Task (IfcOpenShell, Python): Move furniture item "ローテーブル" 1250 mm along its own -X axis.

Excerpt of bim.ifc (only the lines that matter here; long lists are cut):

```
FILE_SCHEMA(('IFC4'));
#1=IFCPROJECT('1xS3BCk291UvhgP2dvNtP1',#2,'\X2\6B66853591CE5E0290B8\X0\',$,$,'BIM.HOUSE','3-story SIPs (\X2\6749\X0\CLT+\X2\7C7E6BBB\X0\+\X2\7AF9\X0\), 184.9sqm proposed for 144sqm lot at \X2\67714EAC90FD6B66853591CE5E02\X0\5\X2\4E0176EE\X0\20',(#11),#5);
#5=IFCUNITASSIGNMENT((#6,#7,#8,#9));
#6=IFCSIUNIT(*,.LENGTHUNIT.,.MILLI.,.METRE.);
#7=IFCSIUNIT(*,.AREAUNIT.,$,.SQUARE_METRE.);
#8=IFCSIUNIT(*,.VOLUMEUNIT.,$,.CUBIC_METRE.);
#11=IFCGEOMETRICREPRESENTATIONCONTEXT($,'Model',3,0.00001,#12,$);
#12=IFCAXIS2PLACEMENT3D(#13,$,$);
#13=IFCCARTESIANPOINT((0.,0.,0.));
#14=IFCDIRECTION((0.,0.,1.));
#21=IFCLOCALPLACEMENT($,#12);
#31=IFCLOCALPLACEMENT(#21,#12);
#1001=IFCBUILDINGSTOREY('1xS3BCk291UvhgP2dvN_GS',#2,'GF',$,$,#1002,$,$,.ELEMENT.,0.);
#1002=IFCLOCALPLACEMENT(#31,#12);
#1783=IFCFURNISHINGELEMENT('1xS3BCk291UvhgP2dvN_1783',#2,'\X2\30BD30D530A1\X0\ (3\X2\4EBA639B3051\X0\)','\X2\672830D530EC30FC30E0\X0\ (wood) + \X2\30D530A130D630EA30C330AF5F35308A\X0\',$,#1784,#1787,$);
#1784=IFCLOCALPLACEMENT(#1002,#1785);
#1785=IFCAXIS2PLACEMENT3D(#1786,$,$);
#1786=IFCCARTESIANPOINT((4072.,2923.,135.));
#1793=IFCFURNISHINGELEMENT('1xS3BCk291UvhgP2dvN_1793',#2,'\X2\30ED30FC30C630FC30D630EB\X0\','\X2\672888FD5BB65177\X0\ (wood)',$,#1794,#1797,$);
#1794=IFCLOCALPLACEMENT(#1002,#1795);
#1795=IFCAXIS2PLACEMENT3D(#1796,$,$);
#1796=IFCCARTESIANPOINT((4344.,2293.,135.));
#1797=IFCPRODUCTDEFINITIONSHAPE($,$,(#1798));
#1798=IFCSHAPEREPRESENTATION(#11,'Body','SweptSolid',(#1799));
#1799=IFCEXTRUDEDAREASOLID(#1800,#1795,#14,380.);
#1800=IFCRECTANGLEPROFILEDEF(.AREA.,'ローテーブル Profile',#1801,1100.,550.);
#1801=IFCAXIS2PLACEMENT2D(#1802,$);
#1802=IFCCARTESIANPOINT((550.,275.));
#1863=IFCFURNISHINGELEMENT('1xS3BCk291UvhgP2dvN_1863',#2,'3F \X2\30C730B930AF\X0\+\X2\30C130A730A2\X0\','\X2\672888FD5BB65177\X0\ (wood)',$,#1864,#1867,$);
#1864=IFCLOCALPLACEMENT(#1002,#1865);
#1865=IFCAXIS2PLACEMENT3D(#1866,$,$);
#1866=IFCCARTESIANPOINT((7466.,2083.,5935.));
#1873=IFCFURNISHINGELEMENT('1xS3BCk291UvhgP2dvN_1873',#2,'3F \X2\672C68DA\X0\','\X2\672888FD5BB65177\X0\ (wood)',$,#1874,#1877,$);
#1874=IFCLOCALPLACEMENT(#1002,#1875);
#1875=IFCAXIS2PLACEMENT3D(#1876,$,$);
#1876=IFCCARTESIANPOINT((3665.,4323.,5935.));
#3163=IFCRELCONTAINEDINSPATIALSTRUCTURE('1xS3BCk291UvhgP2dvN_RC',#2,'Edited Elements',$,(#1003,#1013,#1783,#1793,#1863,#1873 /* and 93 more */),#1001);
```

```python
import ifcopenshell
import ifcopenshell.api.geometry
import ifcopenshell.util.placement
import ifcopenshell.util.unit

model = ifcopenshell.open("bim.ifc")
unit_scale = ifcopenshell.util.unit.calculate_unit_scale(model)

item = model.by_guid("1xS3BCk291UvhgP2dvN_1793")
matrix = ifcopenshell.util.placement.get_local_placement(item.ObjectPlacement)
matrix[:3, 3] -= matrix[:3, 0] * 1.25 / unit_scale
ifcopenshell.api.geometry.edit_object_placement(model, product=item, matrix=matrix, is_si=False)

print(ifcopenshell.util.placement.get_local_placement(item.ObjectPlacement).round(3) + 0.0)

model.write("bim_v2.ifc")
```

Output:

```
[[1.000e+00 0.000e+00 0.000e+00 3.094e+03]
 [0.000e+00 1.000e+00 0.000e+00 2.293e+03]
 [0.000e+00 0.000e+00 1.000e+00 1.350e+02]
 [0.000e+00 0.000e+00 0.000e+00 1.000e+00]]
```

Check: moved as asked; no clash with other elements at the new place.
